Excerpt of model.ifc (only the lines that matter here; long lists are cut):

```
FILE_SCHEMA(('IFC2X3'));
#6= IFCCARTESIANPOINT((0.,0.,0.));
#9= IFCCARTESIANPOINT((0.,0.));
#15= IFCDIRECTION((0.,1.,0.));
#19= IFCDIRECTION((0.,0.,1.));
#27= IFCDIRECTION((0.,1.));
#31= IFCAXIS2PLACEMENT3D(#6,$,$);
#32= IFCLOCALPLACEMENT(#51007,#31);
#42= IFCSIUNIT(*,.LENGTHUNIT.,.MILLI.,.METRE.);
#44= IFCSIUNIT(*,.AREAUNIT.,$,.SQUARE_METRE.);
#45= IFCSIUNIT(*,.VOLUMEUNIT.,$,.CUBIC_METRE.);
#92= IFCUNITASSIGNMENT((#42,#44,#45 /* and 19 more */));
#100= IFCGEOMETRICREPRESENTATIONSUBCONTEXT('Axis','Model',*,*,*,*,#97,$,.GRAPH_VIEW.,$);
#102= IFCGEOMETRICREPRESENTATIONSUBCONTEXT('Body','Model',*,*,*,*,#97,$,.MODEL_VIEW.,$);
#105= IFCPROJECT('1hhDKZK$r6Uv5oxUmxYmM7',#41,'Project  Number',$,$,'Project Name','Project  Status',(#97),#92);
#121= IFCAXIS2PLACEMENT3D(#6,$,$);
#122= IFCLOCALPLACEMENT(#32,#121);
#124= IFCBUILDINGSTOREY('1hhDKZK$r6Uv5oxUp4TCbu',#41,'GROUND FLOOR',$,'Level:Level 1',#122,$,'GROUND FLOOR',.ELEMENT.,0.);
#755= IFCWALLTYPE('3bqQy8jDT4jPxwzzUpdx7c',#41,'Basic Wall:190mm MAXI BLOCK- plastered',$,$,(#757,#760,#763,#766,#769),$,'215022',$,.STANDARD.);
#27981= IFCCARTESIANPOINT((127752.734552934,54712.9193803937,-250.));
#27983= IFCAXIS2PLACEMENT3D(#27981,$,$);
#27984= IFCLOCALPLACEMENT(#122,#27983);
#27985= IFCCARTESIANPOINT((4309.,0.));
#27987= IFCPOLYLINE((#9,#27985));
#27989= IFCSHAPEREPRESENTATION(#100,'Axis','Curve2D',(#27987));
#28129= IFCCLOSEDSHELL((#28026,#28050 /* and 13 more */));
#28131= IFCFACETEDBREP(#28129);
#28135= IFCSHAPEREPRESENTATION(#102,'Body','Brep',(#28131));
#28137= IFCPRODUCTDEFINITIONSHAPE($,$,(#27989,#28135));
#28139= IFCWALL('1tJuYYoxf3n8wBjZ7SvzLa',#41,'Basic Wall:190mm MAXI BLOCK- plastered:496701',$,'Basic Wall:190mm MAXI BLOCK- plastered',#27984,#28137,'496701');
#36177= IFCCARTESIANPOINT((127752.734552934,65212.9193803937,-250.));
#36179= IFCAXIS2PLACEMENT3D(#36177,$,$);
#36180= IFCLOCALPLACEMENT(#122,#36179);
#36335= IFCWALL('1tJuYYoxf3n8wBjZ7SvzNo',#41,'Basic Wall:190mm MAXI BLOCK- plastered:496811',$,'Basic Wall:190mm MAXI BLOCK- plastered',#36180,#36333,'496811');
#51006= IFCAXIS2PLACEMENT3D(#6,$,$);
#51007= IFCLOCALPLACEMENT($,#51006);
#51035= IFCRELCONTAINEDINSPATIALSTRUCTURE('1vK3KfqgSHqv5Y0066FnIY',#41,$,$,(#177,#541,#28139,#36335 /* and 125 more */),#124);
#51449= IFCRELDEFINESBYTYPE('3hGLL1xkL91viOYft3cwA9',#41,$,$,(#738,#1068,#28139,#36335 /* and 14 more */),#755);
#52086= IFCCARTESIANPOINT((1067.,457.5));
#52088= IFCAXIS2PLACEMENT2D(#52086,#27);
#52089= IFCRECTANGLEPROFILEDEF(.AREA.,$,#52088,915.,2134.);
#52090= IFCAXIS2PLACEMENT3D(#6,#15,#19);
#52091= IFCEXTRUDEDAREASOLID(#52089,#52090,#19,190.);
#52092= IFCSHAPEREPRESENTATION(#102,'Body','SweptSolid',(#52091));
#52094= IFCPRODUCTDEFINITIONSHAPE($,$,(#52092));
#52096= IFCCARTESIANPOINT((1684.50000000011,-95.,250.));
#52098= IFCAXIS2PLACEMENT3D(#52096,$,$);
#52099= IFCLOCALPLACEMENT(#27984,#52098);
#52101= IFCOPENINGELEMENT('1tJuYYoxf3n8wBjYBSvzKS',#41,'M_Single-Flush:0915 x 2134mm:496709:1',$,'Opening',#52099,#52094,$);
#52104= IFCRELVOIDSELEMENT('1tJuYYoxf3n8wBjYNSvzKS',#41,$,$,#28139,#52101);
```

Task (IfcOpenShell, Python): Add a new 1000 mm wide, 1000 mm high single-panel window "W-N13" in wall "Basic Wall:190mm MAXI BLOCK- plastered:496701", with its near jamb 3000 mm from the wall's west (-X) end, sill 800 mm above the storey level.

```python
import numpy as np
import ifcopenshell
import ifcopenshell.api.feature
import ifcopenshell.api.geometry
import ifcopenshell.api.root
import ifcopenshell.api.spatial
import ifcopenshell.api.type
import ifcopenshell.geom
import ifcopenshell.util.element
import ifcopenshell.util.placement
import ifcopenshell.util.representation
import ifcopenshell.util.shape
import ifcopenshell.util.unit

model = ifcopenshell.open("model.ifc")
unit_scale = ifcopenshell.util.unit.calculate_unit_scale(model)
settings = ifcopenshell.geom.settings()


def volume(element):
    """Net volume in cubic metres, openings subtracted."""
    shape = ifcopenshell.geom.create_shape(settings, element)
    return ifcopenshell.util.shape.get_volume(shape.geometry)


wall = model.by_guid("1tJuYYoxf3n8wBjZ7SvzLa")
storey = ifcopenshell.util.element.get_container(wall, ifc_class="IfcBuildingStorey")
context = ifcopenshell.util.representation.get_context(model, "Model", "Body", "MODEL_VIEW")
before = volume(wall)

width, height, from_end, sill = 1, 1, 3, 0.8  # metres

# The wall runs along its own X axis, and the end named is its -X end.
wall_shape = ifcopenshell.geom.create_shape(settings, wall)
x, y, z = ifcopenshell.util.shape.get_vertices(wall_shape.geometry).T
start = x.min() + from_end
face, thickness = float(y.min()), float(y.max() - y.min())
wall_matrix = ifcopenshell.util.placement.get_local_placement(wall.ObjectPlacement)
level = ifcopenshell.util.placement.get_local_placement(storey.ObjectPlacement)[2, 3]


def in_wall(x, y):
    """Placement at x, y metres in the wall's axes, at sill height."""
    matrix = wall_matrix.copy()
    matrix[:, 3] = wall_matrix @ np.array([x / unit_scale, y / unit_scale, 0.0, 1.0])
    matrix[2, 3] = level + sill / unit_scale
    return matrix


# Opening: a box that overshoots both wall faces by 50 mm.
opening = ifcopenshell.api.root.create_entity(model, ifc_class="IfcOpeningElement")
box = ifcopenshell.api.geometry.add_wall_representation(
    model, context=context, length=width, height=height, thickness=thickness + 0.1
)
ifcopenshell.api.geometry.assign_representation(model, product=opening, representation=box)
ifcopenshell.api.geometry.edit_object_placement(model, product=opening, matrix=in_wall(start, face - 0.05), is_si=False)
ifcopenshell.api.feature.add_feature(model, feature=opening, element=wall)

window = ifcopenshell.api.root.create_entity(model, ifc_class="IfcWindow", name="W-N13")
window.OverallWidth, window.OverallHeight = width / unit_scale, height / unit_scale
body = ifcopenshell.api.geometry.add_window_representation(
    model,
    context=context,
    overall_width=window.OverallWidth,
    overall_height=window.OverallHeight,
    partition_type="SINGLE_PANEL",
)
ifcopenshell.api.geometry.assign_representation(model, product=window, representation=body)
ifcopenshell.api.spatial.assign_container(model, products=[window], relating_structure=storey)
fills = ifcopenshell.api.feature.add_filling(model, opening=opening, element=window)
fills.OwnerHistory = window.OwnerHistory  # required in IFC2X3

# IFC2X3 keeps the operation on the window style.
style = ifcopenshell.api.root.create_entity(model, ifc_class="IfcWindowStyle", name="W-N13")
style.OperationType, style.ConstructionType = "SINGLE_PANEL", "NOTDEFINED"
style.ParameterTakesPrecedence = style.Sizeable = False
ifcopenshell.api.type.assign_type(model, related_objects=[window], relating_type=style)

# Centre the window in the wall's thickness.
ifcopenshell.api.geometry.edit_object_placement(model, product=window, matrix=in_wall(start, face), is_si=False)
window_shape = ifcopenshell.geom.create_shape(settings, window)
depth = ifcopenshell.util.shape.get_vertices(window_shape.geometry)[:, 1]
offset = face + thickness / 2 - (depth.min() + depth.max()) / 2
ifcopenshell.api.geometry.edit_object_placement(model, product=window, matrix=in_wall(start, offset), is_si=False)

after = volume(wall)

print(f"wall volume {before:.3f} -> {after:.3f} m3")

model.write("model_rev.ifc")
```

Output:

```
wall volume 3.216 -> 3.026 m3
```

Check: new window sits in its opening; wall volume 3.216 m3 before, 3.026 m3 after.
